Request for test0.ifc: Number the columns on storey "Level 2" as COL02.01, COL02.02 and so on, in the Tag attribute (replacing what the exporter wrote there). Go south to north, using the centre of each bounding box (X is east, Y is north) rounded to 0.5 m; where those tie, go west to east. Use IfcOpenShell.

First a look at what the model holds.

```python
import ifcopenshell
import ifcopenshell.util.element
import ifcopenshell.util.placement

model = ifcopenshell.open("test0.ifc")
print(model.schema)
storey = next(s for s in model.by_type("IfcBuildingStorey") if s.Name == "Level 2")
columns = [e for e in ifcopenshell.util.element.get_decomposition(storey) if e.is_a("IfcColumn")]
for e in sorted(columns, key=lambda e: e.id()):
    origin = ifcopenshell.util.placement.get_local_placement(e.ObjectPlacement)[:3, 3]
    print(e.id(), e.Tag, e.Name, origin.round(2) + 0.0, sep=" | ")
```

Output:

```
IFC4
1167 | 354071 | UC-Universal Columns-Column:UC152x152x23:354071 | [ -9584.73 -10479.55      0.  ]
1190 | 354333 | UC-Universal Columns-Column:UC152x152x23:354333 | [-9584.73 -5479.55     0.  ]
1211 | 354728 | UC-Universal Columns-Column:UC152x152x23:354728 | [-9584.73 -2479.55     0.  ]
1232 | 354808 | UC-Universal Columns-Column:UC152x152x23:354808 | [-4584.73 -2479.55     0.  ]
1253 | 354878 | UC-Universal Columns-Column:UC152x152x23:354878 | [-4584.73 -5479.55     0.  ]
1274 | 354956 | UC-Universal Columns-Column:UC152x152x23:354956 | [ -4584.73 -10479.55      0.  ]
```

```python
import ifcopenshell
import ifcopenshell.geom
import ifcopenshell.util.element
import ifcopenshell.util.shape

model = ifcopenshell.open("test0.ifc")
settings = ifcopenshell.geom.settings()
settings.set("use-world-coords", True)


def centre(element):
    shape = ifcopenshell.geom.create_shape(settings, element)
    return ifcopenshell.util.shape.get_bbox_centroid(shape.geometry)


storey = next(s for s in model.by_type("IfcBuildingStorey") if s.Name == "Level 2")
columns = [e for e in ifcopenshell.util.element.get_decomposition(storey) if e.is_a("IfcColumn")]

# Insertion points can sit at a corner or the storey origin, so sort by the geometry (in metres).
centres = {e: centre(e) for e in columns}
columns.sort(key=lambda e: (round(centres[e][1] / 0.5), centres[e][0]))

for i, e in enumerate(columns, start=1):
    number = f"COL02.{i:02d}"
    e.Tag = number
    print(e.id(), number)

model.write("test0-out.ifc")
```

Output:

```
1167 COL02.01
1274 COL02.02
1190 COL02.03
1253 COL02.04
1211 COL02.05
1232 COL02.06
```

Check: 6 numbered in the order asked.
